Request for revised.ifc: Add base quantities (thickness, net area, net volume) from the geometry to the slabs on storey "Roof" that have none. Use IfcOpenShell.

First a look at what the model holds.

```python
import ifcopenshell
import ifcopenshell.util.element
import ifcopenshell.util.unit

model = ifcopenshell.open("revised.ifc")
print(model.schema)
for unit_type in ("LENGTHUNIT", "AREAUNIT", "VOLUMEUNIT"):
    print(unit_type, ifcopenshell.util.unit.calculate_unit_scale(model, unit_type))
storey = next(s for s in model.by_type("IfcBuildingStorey") if s.Name == "Roof")
slabs = [e for e in ifcopenshell.util.element.get_decomposition(storey) if e.is_a("IfcSlab")]
for e in sorted(slabs, key=lambda e: e.id()):
    print(e.id(), e.is_a(), e.Name, list(ifcopenshell.util.element.get_psets(e, qtos_only=True)), sep=" | ")
```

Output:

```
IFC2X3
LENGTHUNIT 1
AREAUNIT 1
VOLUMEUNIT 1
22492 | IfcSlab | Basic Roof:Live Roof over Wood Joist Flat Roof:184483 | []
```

```python
import ifcopenshell
import ifcopenshell.api.pset
import ifcopenshell.geom
import ifcopenshell.util.element
import ifcopenshell.util.shape
import ifcopenshell.util.unit

model = ifcopenshell.open("revised.ifc")
unit_scale = ifcopenshell.util.unit.calculate_unit_scale(model)
area_scale = ifcopenshell.util.unit.calculate_unit_scale(model, "AREAUNIT")
volume_scale = ifcopenshell.util.unit.calculate_unit_scale(model, "VOLUMEUNIT")
settings = ifcopenshell.geom.settings()

storey = next(s for s in model.by_type("IfcBuildingStorey") if s.Name == "Roof")
slabs = [e for e in ifcopenshell.util.element.get_decomposition(storey) if e.is_a("IfcSlab")]

for e in sorted(slabs, key=lambda e: e.id()):
    if ifcopenshell.util.element.get_psets(e, qtos_only=True, should_inherit=False):
        continue
    # Geometry comes back in metres, in the element's own axes.
    shape = ifcopenshell.geom.create_shape(settings, e)
    values = {
        "Width": ifcopenshell.util.shape.get_z(shape.geometry) / unit_scale,
        "NetArea": ifcopenshell.util.shape.get_footprint_area(shape.geometry) / area_scale,
        "NetVolume": ifcopenshell.util.shape.get_volume(shape.geometry) / volume_scale,
    }
    qto = ifcopenshell.api.pset.add_qto(model, product=e, name="BaseQuantities")
    ifcopenshell.api.pset.edit_qto(model, qto=qto, properties=values)
    print(e.id(), {k: round(v, 3) for k, v in values.items()})

model.write("revised_edited.ifc")
```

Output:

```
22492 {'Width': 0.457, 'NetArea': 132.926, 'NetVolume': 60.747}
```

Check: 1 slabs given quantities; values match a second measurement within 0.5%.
